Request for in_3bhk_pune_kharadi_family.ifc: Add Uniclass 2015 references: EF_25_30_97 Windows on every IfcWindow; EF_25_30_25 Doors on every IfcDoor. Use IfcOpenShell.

First a look at what the model holds.

```python
import ifcopenshell

model = ifcopenshell.open("in_3bhk_pune_kharadi_family.ifc")
print(model.schema)
print("classifications:", [c.Name for c in model.by_type("IfcClassification")])
for ifc_class in ("IfcDoor", "IfcRoof", "IfcStair", "IfcWall", "IfcWindow"):
    print(ifc_class, len(model.by_type(ifc_class)))
```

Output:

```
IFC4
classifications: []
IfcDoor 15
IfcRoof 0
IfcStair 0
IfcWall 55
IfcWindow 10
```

```python
import ifcopenshell
import ifcopenshell.api.classification

model = ifcopenshell.open("in_3bhk_pune_kharadi_family.ifc")

system = ifcopenshell.api.classification.add_classification(model, classification="Uniclass 2015")

codes = {
    "IfcWindow": ("EF_25_30_97", "Windows"),
    "IfcDoor": ("EF_25_30_25", "Doors"),
}
for ifc_class, (code, name) in codes.items():
    products = model.by_type(ifc_class)
    ifcopenshell.api.classification.add_reference(
        model, products=products, classification=system, identification=code, name=name
    )
    print(code, len(products))

model.write("in_3bhk_pune_kharadi_family_v2.ifc")
```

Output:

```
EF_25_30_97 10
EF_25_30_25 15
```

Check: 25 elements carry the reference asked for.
